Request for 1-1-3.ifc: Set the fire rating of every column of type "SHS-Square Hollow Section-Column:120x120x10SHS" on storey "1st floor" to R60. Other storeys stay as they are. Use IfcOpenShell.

First a look at what the model holds.

```python
import ifcopenshell
import ifcopenshell.util.element

model = ifcopenshell.open("1-1-3.ifc")
print(model.schema)
storey = next(s for s in model.by_type("IfcBuildingStorey") if s.Name == "1st floor")
columns = [e for e in ifcopenshell.util.element.get_decomposition(storey) if e.is_a("IfcColumn")]
seen = {}
for e in columns:
    element_type = ifcopenshell.util.element.get_type(e)
    key = (element_type.Name if element_type != e and element_type else None, ifcopenshell.util.element.get_pset(e, "Pset_ColumnCommon", "FireRating"))
    seen[key] = seen.get(key, 0) + 1
for (name, value), count in sorted(seen.items(), key=str):
    print(count, "x", name, "|", value)
```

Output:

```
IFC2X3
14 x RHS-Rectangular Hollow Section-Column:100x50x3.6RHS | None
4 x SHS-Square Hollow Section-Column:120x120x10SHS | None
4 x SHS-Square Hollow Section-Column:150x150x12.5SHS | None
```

```python
import ifcopenshell
import ifcopenshell.api.pset
import ifcopenshell.util.element

model = ifcopenshell.open("1-1-3.ifc")

storey = next(s for s in model.by_type("IfcBuildingStorey") if s.Name == "1st floor")
columns = [e for e in ifcopenshell.util.element.get_decomposition(storey) if e.is_a("IfcColumn")]

count = 0
for e in columns:
    element_type = ifcopenshell.util.element.get_type(e)
    if element_type in (None, e) or element_type.Name != "SHS-Square Hollow Section-Column:120x120x10SHS":
        continue
    # add_pset returns the element's existing set when there is one.
    pset = ifcopenshell.api.pset.add_pset(model, product=e, name="Pset_ColumnCommon")
    ifcopenshell.api.pset.edit_pset(model, pset=pset, properties={"FireRating": "R60"})
    count += 1

print(count, "columns updated")

model.write("1-1-3_rev.ifc")
```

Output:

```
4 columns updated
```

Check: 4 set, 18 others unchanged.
